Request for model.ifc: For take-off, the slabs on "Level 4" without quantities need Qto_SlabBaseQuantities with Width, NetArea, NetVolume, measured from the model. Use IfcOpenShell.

First a look at what the model holds.

```python
import ifcopenshell
import ifcopenshell.util.element
import ifcopenshell.util.unit

model = ifcopenshell.open("model.ifc")
print(model.schema)
for unit_type in ("LENGTHUNIT", "AREAUNIT", "VOLUMEUNIT"):
    print(unit_type, ifcopenshell.util.unit.calculate_unit_scale(model, unit_type))
storey = next(s for s in model.by_type("IfcBuildingStorey") if s.Name == "Level 4")
slabs = [e for e in ifcopenshell.util.element.get_decomposition(storey) if e.is_a("IfcSlab")]
for e in sorted(slabs, key=lambda e: e.id()):
    print(e.id(), e.is_a(), e.Name, list(ifcopenshell.util.element.get_psets(e, qtos_only=True)), sep=" | ")
```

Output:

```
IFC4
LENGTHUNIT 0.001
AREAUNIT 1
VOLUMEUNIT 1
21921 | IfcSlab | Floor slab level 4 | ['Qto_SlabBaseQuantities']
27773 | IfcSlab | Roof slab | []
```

```python
import ifcopenshell
import ifcopenshell.api.pset
import ifcopenshell.geom
import ifcopenshell.util.element
import ifcopenshell.util.shape
import ifcopenshell.util.unit

model = ifcopenshell.open("model.ifc")
unit_scale = ifcopenshell.util.unit.calculate_unit_scale(model)
area_scale = ifcopenshell.util.unit.calculate_unit_scale(model, "AREAUNIT")
volume_scale = ifcopenshell.util.unit.calculate_unit_scale(model, "VOLUMEUNIT")
settings = ifcopenshell.geom.settings()

storey = next(s for s in model.by_type("IfcBuildingStorey") if s.Name == "Level 4")
slabs = [e for e in ifcopenshell.util.element.get_decomposition(storey) if e.is_a("IfcSlab")]

for e in sorted(slabs, key=lambda e: e.id()):
    if ifcopenshell.util.element.get_psets(e, qtos_only=True, should_inherit=False):
        continue
    # Geometry comes back in metres, in the element's own axes.
    shape = ifcopenshell.geom.create_shape(settings, e)
    values = {
        "Width": ifcopenshell.util.shape.get_z(shape.geometry) / unit_scale,
        "NetArea": ifcopenshell.util.shape.get_footprint_area(shape.geometry) / area_scale,
        "NetVolume": ifcopenshell.util.shape.get_volume(shape.geometry) / volume_scale,
    }
    qto = ifcopenshell.api.pset.add_qto(model, product=e, name="Qto_SlabBaseQuantities")
    ifcopenshell.api.pset.edit_qto(model, qto=qto, properties=values)
    print(e.id(), {k: round(v, 3) for k, v in values.items()})

model.write("model_edited.ifc")
```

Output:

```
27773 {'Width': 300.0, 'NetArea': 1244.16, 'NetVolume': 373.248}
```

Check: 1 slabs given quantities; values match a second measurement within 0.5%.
